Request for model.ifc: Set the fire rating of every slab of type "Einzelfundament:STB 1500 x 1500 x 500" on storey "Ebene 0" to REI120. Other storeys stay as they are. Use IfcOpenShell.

First a look at what the model holds.

```python
import ifcopenshell
import ifcopenshell.util.element

model = ifcopenshell.open("model.ifc")
print(model.schema)
storey = next(s for s in model.by_type("IfcBuildingStorey") if s.Name == "Ebene 0")
slabs = [e for e in ifcopenshell.util.element.get_decomposition(storey) if e.is_a("IfcSlab")]
seen = {}
for e in slabs:
    element_type = ifcopenshell.util.element.get_type(e)
    key = (element_type.Name if element_type != e and element_type else None, ifcopenshell.util.element.get_pset(e, "Pset_SlabCommon", "FireRating"))
    seen[key] = seen.get(key, 0) + 1
for (name, value), count in sorted(seen.items(), key=str):
    print(count, "x", name, "|", value)
```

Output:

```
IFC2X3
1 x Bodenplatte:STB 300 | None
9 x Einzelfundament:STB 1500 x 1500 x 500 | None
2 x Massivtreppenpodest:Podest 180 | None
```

```python
import ifcopenshell
import ifcopenshell.api.pset
import ifcopenshell.util.element

model = ifcopenshell.open("model.ifc")

storey = next(s for s in model.by_type("IfcBuildingStorey") if s.Name == "Ebene 0")
slabs = [e for e in ifcopenshell.util.element.get_decomposition(storey) if e.is_a("IfcSlab")]

count = 0
for e in slabs:
    element_type = ifcopenshell.util.element.get_type(e)
    if element_type in (None, e) or element_type.Name != "Einzelfundament:STB 1500 x 1500 x 500":
        continue
    # add_pset returns the element's existing set when there is one.
    pset = ifcopenshell.api.pset.add_pset(model, product=e, name="Pset_SlabCommon")
    ifcopenshell.api.pset.edit_pset(model, pset=pset, properties={"FireRating": "REI120"})
    count += 1

print(count, "slabs updated")

model.write("model_v2.ifc")
```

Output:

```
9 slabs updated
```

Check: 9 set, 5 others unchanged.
